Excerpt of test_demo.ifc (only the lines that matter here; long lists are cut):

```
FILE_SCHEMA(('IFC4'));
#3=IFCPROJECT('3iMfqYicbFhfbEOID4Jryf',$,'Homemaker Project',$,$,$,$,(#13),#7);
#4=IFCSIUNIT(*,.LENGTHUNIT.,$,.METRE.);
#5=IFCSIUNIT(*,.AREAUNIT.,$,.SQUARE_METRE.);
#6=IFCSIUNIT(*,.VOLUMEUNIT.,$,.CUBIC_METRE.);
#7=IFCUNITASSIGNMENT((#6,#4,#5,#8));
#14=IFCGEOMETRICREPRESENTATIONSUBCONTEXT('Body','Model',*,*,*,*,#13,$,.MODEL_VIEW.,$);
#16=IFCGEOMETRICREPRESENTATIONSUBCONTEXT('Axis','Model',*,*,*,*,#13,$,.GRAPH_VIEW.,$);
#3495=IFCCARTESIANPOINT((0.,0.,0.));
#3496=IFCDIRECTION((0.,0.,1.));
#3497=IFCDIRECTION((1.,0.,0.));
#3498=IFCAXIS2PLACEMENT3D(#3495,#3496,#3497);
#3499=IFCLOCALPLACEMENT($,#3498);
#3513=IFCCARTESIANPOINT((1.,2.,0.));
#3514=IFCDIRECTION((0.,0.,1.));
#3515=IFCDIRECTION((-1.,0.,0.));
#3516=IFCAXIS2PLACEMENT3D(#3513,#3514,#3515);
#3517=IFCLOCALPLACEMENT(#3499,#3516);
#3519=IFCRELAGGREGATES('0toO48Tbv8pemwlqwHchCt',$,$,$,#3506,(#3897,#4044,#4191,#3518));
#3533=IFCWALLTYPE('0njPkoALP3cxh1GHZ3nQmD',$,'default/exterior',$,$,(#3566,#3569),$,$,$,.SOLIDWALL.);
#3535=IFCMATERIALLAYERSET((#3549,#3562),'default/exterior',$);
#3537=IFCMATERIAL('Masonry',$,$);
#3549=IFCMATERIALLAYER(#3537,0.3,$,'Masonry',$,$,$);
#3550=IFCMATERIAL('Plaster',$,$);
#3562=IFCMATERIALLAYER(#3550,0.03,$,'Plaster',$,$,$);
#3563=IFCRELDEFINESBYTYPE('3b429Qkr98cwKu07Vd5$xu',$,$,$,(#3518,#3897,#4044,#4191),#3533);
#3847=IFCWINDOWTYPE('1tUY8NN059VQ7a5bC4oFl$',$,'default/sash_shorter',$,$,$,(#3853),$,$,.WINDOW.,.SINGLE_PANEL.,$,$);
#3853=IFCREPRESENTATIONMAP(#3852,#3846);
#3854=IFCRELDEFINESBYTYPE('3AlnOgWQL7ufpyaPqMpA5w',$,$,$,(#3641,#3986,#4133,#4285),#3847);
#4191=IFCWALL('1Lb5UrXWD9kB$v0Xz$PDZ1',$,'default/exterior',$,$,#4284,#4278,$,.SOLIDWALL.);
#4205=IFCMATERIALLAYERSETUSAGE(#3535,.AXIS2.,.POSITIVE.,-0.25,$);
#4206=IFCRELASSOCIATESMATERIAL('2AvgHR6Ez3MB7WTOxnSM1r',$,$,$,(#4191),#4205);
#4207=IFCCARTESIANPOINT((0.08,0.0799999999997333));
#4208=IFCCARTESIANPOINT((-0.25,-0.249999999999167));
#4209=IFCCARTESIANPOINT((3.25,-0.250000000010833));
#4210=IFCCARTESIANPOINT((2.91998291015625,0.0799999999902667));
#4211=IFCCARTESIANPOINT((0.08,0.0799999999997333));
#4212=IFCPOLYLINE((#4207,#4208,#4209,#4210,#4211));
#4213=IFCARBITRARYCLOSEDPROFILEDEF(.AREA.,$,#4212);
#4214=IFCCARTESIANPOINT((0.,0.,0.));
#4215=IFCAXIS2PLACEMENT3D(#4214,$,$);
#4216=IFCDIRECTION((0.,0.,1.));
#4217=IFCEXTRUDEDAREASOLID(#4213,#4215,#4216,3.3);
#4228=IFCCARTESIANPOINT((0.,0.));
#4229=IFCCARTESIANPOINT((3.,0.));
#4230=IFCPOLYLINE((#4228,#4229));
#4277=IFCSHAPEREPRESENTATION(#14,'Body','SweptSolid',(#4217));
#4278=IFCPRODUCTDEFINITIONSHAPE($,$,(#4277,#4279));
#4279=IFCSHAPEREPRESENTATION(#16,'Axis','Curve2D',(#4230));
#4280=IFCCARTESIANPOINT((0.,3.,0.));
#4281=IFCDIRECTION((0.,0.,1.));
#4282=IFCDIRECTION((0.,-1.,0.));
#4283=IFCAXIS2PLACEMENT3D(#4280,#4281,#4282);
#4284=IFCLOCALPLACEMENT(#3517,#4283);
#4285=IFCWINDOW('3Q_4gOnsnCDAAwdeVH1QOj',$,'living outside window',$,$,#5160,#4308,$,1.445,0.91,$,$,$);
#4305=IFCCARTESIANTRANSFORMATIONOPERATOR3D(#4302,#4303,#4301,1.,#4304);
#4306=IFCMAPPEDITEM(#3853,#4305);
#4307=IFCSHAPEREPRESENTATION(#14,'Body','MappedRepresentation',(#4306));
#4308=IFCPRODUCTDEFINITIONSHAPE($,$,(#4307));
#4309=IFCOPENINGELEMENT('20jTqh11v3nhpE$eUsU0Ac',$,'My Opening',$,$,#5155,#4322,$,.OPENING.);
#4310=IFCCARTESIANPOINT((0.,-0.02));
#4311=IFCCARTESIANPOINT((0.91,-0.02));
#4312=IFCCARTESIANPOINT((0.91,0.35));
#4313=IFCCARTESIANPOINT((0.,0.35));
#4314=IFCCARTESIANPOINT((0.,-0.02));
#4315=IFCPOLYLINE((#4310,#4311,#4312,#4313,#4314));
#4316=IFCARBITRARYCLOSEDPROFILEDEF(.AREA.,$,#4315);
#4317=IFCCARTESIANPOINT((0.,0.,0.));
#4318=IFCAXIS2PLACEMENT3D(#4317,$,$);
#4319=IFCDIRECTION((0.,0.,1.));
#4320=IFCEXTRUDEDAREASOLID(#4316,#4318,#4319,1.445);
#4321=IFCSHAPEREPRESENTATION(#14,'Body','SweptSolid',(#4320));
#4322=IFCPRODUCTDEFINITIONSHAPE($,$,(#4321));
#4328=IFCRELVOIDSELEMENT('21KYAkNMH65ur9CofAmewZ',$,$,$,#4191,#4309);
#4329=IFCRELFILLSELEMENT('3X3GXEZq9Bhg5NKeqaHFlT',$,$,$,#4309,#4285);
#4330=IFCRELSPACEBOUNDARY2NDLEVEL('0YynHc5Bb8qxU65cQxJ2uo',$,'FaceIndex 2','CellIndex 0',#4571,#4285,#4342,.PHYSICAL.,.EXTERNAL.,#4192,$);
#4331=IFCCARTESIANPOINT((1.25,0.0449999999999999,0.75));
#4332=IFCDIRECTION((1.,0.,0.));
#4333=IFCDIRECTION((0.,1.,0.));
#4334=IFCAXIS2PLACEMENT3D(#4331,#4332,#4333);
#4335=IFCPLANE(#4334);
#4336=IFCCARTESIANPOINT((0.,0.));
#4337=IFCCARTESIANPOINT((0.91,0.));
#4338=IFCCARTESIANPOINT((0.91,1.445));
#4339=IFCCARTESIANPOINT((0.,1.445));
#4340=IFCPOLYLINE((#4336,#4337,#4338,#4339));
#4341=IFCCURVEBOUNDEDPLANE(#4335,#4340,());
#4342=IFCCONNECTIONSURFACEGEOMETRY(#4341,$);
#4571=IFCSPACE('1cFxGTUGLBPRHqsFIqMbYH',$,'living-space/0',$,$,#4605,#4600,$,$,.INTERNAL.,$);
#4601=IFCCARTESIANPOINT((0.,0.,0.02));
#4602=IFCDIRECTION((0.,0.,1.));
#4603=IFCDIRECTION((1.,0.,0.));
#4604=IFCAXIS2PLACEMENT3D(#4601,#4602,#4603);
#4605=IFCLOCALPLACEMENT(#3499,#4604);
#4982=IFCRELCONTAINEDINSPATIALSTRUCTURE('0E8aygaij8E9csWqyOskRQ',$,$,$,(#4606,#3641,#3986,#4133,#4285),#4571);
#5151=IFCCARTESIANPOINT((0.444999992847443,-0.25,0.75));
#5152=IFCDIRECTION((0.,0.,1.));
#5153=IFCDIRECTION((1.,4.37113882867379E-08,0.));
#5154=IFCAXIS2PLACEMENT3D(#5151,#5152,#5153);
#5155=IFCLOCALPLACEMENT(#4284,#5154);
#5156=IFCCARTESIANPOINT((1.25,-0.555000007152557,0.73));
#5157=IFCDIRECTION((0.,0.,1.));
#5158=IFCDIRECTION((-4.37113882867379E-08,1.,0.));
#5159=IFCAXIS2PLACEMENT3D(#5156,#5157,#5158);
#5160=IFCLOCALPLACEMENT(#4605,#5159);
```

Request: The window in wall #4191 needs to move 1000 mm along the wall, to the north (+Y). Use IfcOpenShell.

```python
import numpy as np
import ifcopenshell
import ifcopenshell.api.geometry
import ifcopenshell.util.placement
import ifcopenshell.util.unit

model = ifcopenshell.open("test_demo.ifc")
unit_scale = ifcopenshell.util.unit.calculate_unit_scale(model)

window = model.by_id(4285)
opening = window.FillsVoids[0].RelatingOpeningElement
wall = opening.VoidsElements[0].RelatingBuildingElement

wall_matrix = ifcopenshell.util.placement.get_local_placement(wall.ObjectPlacement)
shift = wall_matrix[:3, 0] * 1 / unit_scale
before = ifcopenshell.util.placement.get_local_placement(window.ObjectPlacement)[:3, 3].copy()

# The window is not placed relative to its opening, so move both.
for product in (opening, window):
    matrix = ifcopenshell.util.placement.get_local_placement(product.ObjectPlacement)
    matrix[:3, 3] += shift
    ifcopenshell.api.geometry.edit_object_placement(model, product=product, matrix=matrix, is_si=False)

# Space boundary surfaces are stored in each space's coordinates; move them too.
for rel in window.ProvidesBoundaries:
    if not rel.ConnectionGeometry:
        continue
    surface = rel.ConnectionGeometry.SurfaceOnRelatingElement.BasisSurface
    space_matrix = ifcopenshell.util.placement.get_local_placement(rel.RelatingSpace.ObjectPlacement)
    point = np.array(surface.Position.Location.Coordinates) + space_matrix[:3, :3].T @ shift
    surface.Position = model.createIfcAxis2Placement3D(
        model.createIfcCartesianPoint(point.tolist()), surface.Position.Axis, surface.Position.RefDirection
    )

after = ifcopenshell.util.placement.get_local_placement(window.ObjectPlacement)[:3, 3]
print("window moved by", (after - before).round(3) + 0.0)

model.write("test_demo_updated.ifc")
```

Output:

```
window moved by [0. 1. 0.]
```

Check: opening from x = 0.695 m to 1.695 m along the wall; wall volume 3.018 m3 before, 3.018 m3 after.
